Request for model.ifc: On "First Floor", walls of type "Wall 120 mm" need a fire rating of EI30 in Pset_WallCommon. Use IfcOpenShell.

First a look at what the model holds.

```python
import ifcopenshell
import ifcopenshell.util.element

model = ifcopenshell.open("model.ifc")
print(model.schema)
storey = next(s for s in model.by_type("IfcBuildingStorey") if s.Name == "First Floor")
walls = [e for e in ifcopenshell.util.element.get_decomposition(storey) if e.is_a("IfcWall")]
seen = {}
for e in walls:
    element_type = ifcopenshell.util.element.get_type(e)
    key = (element_type.Name if element_type != e and element_type else None, ifcopenshell.util.element.get_pset(e, "Pset_WallCommon", "FireRating"))
    seen[key] = seen.get(key, 0) + 1
for (name, value), count in sorted(seen.items(), key=str):
    print(count, "x", name, "|", value)
```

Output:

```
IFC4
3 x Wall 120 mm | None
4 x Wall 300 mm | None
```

```python
import ifcopenshell
import ifcopenshell.api.pset
import ifcopenshell.util.element

model = ifcopenshell.open("model.ifc")

storey = next(s for s in model.by_type("IfcBuildingStorey") if s.Name == "First Floor")
walls = [e for e in ifcopenshell.util.element.get_decomposition(storey) if e.is_a("IfcWall")]

count = 0
for e in walls:
    element_type = ifcopenshell.util.element.get_type(e)
    if element_type in (None, e) or element_type.Name != "Wall 120 mm":
        continue
    # add_pset returns the element's existing set when there is one.
    pset = ifcopenshell.api.pset.add_pset(model, product=e, name="Pset_WallCommon")
    ifcopenshell.api.pset.edit_pset(model, pset=pset, properties={"FireRating": "EI30"})
    count += 1

print(count, "walls updated")

model.write("model_v2.ifc")
```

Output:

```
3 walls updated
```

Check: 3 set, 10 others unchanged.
